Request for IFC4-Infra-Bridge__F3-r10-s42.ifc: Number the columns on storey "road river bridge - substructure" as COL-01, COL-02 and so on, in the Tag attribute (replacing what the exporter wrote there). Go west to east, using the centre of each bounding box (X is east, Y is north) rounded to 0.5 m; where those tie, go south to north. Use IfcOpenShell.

First a look at what the model holds.

```python
import ifcopenshell
import ifcopenshell.util.element
import ifcopenshell.util.placement

model = ifcopenshell.open("IFC4-Infra-Bridge__F3-r10-s42.ifc")
print(model.schema)
storey = next(s for s in model.by_type("IfcBuildingStorey") if s.Name == "road river bridge - substructure")
columns = [e for e in ifcopenshell.util.element.get_decomposition(storey) if e.is_a("IfcColumn")]
for e in sorted(columns, key=lambda e: e.id()):
    origin = ifcopenshell.util.placement.get_local_placement(e.ObjectPlacement)[:3, 3]
    print(e.id(), e.Tag, e.Name, origin.round(2) + 0.0, sep=" | ")
```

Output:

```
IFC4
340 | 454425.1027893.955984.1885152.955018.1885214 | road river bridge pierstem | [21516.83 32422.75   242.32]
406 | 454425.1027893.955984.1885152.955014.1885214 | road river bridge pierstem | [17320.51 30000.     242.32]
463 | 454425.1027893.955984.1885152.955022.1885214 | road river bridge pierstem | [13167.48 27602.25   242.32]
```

```python
import ifcopenshell
import ifcopenshell.geom
import ifcopenshell.util.element
import ifcopenshell.util.shape

model = ifcopenshell.open("IFC4-Infra-Bridge__F3-r10-s42.ifc")
settings = ifcopenshell.geom.settings()
settings.set("use-world-coords", True)


def centre(element):
    shape = ifcopenshell.geom.create_shape(settings, element)
    return ifcopenshell.util.shape.get_bbox_centroid(shape.geometry)


storey = next(s for s in model.by_type("IfcBuildingStorey") if s.Name == "road river bridge - substructure")
columns = [e for e in ifcopenshell.util.element.get_decomposition(storey) if e.is_a("IfcColumn")]

# Insertion points can sit at a corner or the storey origin, so sort by the geometry (in metres).
centres = {e: centre(e) for e in columns}
columns.sort(key=lambda e: (round(centres[e][0] / 0.5), centres[e][1]))

for i, e in enumerate(columns, start=1):
    number = f"COL-{i:02d}"
    e.Tag = number
    print(e.id(), number)

model.write("IFC4-Infra-Bridge__F3-r10-s42_edited.ifc")
```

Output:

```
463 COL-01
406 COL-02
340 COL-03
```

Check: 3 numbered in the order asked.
